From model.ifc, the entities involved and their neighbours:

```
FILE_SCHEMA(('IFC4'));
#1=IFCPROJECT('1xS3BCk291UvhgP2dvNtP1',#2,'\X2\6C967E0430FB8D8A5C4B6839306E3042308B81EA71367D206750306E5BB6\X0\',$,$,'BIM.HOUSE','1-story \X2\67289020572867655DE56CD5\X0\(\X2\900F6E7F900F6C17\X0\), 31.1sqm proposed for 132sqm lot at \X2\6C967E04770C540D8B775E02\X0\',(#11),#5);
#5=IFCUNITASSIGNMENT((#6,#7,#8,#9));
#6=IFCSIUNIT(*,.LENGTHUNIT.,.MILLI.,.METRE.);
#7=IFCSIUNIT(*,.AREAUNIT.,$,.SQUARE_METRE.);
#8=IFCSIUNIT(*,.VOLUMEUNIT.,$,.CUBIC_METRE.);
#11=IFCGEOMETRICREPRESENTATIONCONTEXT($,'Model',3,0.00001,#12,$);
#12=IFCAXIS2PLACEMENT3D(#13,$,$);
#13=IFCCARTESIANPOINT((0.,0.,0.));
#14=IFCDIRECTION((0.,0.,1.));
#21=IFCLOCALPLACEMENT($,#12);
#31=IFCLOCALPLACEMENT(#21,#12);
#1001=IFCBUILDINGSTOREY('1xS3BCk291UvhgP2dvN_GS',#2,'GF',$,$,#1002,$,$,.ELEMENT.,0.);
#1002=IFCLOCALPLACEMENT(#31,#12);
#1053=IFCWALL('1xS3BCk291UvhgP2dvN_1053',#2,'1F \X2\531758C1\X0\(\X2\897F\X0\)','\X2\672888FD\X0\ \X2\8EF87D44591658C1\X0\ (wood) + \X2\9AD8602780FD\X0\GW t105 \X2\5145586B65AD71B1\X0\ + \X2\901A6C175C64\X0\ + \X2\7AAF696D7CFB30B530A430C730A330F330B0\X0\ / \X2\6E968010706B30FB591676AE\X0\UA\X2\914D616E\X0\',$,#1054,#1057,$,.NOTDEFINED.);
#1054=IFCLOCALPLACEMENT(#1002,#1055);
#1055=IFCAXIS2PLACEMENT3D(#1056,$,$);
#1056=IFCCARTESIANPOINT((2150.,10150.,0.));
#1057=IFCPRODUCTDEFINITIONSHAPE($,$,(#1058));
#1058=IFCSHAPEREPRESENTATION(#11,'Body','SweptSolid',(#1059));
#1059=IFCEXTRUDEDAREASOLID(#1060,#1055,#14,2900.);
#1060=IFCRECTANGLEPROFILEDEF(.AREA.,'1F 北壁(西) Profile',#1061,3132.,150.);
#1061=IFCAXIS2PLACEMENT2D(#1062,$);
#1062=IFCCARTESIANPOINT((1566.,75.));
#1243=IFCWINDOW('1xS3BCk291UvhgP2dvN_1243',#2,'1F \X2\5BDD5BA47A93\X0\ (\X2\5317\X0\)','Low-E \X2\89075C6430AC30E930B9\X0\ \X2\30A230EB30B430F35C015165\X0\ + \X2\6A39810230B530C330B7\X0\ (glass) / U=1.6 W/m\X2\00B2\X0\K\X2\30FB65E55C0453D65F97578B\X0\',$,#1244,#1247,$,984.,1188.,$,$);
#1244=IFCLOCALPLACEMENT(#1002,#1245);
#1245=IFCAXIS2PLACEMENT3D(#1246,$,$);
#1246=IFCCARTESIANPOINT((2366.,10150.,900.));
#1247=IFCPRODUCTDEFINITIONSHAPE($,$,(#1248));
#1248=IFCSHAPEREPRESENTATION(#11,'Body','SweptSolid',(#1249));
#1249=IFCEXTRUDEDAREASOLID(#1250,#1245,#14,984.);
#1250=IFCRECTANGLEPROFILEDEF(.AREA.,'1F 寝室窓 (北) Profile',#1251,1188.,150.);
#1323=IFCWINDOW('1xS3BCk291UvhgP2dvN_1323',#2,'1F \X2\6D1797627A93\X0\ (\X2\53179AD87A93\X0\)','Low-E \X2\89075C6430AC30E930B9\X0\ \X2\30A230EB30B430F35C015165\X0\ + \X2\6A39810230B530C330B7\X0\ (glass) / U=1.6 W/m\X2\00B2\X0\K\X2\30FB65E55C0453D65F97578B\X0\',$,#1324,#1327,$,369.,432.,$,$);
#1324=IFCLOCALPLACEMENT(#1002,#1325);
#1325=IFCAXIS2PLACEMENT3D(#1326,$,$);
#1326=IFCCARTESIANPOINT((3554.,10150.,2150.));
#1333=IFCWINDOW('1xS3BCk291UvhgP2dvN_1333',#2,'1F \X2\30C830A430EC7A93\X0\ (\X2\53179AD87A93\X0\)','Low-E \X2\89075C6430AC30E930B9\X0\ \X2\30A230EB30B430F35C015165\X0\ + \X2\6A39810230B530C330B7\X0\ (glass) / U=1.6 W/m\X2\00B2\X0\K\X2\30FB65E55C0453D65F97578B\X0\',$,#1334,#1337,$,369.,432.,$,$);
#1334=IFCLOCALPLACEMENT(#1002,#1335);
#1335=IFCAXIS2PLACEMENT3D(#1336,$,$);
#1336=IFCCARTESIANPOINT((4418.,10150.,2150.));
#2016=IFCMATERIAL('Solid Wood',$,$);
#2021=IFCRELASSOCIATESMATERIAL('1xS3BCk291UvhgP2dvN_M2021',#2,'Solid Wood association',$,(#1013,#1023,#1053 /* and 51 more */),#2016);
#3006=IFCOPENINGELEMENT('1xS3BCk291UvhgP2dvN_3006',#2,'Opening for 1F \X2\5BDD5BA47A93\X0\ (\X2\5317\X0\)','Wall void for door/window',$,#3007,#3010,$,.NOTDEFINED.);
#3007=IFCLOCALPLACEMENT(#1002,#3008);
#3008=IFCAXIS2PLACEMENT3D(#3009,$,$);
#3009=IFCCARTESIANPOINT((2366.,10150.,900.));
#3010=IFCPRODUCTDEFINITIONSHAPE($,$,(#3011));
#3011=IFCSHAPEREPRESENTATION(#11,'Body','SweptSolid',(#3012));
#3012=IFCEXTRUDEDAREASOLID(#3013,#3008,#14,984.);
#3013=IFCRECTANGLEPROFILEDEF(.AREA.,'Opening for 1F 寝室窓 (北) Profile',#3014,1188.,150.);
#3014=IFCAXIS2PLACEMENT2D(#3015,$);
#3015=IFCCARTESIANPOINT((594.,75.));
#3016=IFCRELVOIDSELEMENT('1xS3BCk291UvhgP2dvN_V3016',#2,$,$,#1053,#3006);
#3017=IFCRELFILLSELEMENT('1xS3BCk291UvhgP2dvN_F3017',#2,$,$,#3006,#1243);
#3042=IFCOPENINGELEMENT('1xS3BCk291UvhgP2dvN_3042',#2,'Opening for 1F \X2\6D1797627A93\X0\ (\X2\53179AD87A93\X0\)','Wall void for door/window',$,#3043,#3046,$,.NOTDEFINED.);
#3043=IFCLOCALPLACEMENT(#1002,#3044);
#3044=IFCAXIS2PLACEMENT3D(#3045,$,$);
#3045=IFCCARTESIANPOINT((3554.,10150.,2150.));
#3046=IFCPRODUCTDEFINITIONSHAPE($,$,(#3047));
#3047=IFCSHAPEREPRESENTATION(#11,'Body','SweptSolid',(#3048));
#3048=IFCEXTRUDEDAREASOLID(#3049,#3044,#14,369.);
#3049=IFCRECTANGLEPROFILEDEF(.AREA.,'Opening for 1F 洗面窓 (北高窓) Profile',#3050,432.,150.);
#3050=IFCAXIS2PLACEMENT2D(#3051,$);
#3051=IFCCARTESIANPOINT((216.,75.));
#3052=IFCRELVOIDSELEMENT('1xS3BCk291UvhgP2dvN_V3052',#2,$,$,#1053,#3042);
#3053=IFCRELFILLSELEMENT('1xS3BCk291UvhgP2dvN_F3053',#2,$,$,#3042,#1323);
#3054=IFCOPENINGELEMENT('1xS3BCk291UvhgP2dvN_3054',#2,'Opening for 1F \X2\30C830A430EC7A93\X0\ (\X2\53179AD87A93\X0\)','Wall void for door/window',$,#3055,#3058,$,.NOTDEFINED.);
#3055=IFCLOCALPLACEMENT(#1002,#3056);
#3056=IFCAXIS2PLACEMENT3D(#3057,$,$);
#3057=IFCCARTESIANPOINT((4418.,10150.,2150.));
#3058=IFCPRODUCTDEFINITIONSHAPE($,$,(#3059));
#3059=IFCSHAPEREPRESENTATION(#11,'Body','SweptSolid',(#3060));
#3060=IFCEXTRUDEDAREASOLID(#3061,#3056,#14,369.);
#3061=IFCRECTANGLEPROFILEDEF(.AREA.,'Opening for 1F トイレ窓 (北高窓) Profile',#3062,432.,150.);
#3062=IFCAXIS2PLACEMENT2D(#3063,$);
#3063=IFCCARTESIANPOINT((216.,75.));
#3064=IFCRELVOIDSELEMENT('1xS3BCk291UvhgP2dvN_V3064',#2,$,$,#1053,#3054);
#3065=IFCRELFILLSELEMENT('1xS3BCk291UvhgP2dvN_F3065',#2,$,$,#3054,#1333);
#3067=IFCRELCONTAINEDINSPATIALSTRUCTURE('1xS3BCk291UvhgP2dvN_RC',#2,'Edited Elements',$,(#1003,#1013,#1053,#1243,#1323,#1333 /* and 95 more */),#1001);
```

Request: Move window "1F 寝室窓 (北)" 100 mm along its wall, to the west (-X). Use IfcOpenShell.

```python
import ifcopenshell
import ifcopenshell.api.geometry
import ifcopenshell.util.placement
import ifcopenshell.util.unit

model = ifcopenshell.open("model.ifc")
unit_scale = ifcopenshell.util.unit.calculate_unit_scale(model)

window = model.by_guid("1xS3BCk291UvhgP2dvN_1243")
opening = window.FillsVoids[0].RelatingOpeningElement
wall = opening.VoidsElements[0].RelatingBuildingElement

wall_matrix = ifcopenshell.util.placement.get_local_placement(wall.ObjectPlacement)
shift = wall_matrix[:3, 0] * -0.1 / unit_scale
before = ifcopenshell.util.placement.get_local_placement(window.ObjectPlacement)[:3, 3].copy()

# The window is not placed relative to its opening, so move both.
for product in (opening, window):
    matrix = ifcopenshell.util.placement.get_local_placement(product.ObjectPlacement)
    matrix[:3, 3] += shift
    ifcopenshell.api.geometry.edit_object_placement(model, product=product, matrix=matrix, is_si=False)

after = ifcopenshell.util.placement.get_local_placement(window.ObjectPlacement)[:3, 3]
print("window moved by", (after - before).round(3) + 0.0)

model.write("model_updated.ifc")
```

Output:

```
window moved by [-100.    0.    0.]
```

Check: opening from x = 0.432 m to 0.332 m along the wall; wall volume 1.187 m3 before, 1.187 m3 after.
